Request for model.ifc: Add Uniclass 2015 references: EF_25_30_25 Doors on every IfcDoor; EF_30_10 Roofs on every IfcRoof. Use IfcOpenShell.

First a look at what the model holds.

```python
import ifcopenshell

model = ifcopenshell.open("model.ifc")
print(model.schema)
print("classifications:", [c.Name for c in model.by_type("IfcClassification")])
for ifc_class in ("IfcDoor", "IfcRoof", "IfcStair", "IfcWall", "IfcWindow"):
    print(ifc_class, len(model.by_type(ifc_class)))
```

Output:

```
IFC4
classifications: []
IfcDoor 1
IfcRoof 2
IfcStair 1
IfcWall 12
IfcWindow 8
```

```python
import ifcopenshell
import ifcopenshell.api.classification

model = ifcopenshell.open("model.ifc")

system = ifcopenshell.api.classification.add_classification(model, classification="Uniclass 2015")

codes = {
    "IfcDoor": ("EF_25_30_25", "Doors"),
    "IfcRoof": ("EF_30_10", "Roofs"),
}
for ifc_class, (code, name) in codes.items():
    products = model.by_type(ifc_class)
    ifcopenshell.api.classification.add_reference(
        model, products=products, classification=system, identification=code, name=name
    )
    print(code, len(products))

model.write("model_updated.ifc")
```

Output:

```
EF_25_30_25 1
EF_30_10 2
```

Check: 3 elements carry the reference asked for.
